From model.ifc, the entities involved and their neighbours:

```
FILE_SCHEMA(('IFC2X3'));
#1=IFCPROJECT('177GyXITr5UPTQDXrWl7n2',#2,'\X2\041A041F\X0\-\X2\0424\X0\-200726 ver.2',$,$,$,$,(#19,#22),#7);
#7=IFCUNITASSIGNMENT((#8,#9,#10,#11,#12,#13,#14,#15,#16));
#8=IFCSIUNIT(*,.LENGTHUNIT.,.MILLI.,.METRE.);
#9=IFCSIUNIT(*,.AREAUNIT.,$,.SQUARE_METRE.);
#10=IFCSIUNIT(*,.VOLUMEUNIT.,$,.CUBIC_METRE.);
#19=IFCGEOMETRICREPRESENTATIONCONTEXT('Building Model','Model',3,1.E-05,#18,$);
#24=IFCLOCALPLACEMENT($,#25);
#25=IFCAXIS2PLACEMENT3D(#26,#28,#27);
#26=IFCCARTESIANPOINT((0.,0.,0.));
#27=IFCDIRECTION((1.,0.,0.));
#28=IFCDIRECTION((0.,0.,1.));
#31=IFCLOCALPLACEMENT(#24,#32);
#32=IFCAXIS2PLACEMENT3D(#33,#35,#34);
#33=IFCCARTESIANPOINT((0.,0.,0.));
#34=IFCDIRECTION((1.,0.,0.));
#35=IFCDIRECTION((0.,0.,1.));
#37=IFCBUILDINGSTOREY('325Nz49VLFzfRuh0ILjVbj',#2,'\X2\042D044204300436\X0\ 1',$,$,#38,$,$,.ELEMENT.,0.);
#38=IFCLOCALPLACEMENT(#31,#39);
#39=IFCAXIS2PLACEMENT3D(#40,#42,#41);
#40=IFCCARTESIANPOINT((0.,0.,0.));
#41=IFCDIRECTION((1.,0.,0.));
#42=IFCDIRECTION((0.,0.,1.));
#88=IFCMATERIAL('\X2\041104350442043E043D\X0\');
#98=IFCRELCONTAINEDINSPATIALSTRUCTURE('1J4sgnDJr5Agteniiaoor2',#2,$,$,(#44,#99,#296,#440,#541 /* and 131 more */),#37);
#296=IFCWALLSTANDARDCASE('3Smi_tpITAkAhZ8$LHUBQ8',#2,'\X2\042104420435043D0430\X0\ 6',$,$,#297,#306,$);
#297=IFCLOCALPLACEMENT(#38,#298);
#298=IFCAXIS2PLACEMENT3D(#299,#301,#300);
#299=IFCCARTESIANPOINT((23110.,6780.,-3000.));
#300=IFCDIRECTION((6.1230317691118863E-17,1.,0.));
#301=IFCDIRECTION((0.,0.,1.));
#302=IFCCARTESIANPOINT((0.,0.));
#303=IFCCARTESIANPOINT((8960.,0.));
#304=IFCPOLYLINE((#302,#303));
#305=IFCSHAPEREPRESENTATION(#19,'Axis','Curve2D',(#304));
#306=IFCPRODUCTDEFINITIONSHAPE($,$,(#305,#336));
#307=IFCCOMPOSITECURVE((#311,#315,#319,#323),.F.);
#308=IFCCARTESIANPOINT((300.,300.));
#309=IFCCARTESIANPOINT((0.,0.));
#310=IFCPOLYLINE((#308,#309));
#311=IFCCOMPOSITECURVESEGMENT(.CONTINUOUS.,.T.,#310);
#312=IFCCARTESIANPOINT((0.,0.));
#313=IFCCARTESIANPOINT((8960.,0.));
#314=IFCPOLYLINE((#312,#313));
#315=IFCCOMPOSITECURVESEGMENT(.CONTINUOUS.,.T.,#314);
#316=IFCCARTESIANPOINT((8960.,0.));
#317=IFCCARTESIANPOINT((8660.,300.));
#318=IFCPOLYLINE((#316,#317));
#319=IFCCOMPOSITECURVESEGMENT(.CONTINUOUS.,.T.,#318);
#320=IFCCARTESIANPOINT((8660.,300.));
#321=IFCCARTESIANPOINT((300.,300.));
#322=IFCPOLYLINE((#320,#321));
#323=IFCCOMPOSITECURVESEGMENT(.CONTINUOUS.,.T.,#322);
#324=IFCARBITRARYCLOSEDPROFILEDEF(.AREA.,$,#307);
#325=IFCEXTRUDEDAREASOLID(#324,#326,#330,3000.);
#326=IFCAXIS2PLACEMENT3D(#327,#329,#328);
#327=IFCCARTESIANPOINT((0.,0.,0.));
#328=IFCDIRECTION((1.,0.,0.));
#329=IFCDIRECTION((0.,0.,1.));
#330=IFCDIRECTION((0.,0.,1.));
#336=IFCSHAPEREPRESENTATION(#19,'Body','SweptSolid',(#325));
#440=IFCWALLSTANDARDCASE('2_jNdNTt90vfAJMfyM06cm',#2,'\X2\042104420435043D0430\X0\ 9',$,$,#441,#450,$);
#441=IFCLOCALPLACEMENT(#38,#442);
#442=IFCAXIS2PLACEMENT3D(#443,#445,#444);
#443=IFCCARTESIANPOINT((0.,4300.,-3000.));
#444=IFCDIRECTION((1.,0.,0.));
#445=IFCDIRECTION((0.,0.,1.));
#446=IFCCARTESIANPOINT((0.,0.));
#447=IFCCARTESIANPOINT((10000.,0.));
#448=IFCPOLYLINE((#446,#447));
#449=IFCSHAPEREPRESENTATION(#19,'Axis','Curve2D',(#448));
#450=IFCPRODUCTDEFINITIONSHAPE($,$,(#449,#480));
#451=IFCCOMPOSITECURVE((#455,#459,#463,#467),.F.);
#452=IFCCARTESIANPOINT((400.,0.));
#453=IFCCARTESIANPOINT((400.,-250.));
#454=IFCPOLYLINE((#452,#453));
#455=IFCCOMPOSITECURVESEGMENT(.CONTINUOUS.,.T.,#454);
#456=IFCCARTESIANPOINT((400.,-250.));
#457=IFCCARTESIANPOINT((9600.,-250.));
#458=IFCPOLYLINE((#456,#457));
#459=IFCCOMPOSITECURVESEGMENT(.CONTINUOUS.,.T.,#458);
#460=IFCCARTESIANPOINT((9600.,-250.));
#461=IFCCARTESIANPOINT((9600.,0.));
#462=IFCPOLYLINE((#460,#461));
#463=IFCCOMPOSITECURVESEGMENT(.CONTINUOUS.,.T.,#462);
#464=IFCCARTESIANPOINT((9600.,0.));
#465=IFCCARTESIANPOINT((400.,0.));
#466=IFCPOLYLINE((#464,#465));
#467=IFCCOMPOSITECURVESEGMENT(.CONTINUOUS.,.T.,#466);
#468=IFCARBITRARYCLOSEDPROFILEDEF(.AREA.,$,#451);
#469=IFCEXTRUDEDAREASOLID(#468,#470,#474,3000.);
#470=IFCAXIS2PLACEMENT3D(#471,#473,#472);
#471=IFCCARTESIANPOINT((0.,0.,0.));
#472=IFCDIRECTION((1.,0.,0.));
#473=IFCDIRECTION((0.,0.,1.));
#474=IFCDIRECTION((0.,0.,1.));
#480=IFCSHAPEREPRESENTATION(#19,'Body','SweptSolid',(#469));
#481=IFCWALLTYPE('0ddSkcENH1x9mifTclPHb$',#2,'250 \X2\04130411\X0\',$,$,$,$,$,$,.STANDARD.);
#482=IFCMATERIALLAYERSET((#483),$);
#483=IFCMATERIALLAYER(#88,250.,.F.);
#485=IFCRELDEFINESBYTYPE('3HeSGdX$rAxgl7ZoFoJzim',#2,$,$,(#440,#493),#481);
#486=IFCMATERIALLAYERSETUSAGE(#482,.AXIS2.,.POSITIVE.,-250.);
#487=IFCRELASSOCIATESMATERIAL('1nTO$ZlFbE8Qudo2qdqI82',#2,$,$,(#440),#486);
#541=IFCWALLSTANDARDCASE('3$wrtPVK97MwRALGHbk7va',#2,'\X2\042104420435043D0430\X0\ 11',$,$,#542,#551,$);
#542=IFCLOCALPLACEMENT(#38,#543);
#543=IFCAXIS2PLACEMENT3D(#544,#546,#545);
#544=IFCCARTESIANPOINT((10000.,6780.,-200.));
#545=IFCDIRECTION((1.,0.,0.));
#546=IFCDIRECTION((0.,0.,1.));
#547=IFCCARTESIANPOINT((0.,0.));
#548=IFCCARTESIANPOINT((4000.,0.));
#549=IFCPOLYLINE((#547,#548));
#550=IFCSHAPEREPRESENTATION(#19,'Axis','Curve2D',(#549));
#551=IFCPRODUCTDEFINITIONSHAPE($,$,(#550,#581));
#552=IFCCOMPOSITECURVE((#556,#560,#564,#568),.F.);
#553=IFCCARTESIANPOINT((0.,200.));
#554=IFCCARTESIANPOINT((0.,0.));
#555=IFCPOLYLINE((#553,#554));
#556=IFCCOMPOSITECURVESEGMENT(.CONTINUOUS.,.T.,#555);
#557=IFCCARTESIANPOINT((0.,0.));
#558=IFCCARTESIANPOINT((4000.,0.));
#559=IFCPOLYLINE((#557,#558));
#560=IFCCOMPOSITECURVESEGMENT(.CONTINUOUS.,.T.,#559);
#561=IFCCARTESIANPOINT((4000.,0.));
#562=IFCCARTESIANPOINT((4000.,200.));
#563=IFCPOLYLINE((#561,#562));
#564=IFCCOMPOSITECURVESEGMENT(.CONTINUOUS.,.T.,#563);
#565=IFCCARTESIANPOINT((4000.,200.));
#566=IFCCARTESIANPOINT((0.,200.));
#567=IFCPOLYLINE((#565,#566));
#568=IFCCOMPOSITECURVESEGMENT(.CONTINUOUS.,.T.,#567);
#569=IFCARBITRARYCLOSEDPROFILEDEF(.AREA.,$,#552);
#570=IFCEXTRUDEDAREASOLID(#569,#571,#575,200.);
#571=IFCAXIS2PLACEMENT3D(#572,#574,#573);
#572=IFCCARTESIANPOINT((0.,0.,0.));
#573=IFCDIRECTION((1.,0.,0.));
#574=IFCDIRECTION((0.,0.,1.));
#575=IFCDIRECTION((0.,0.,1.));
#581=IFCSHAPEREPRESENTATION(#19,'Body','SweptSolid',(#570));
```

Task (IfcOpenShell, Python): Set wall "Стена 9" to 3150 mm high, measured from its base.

```python
import ifcopenshell
import ifcopenshell.geom
import ifcopenshell.util.shape
import ifcopenshell.util.unit

model = ifcopenshell.open("model.ifc")
unit_scale = ifcopenshell.util.unit.calculate_unit_scale(model)
settings = ifcopenshell.geom.settings()


def volume(element):
    """Net volume in cubic metres, openings subtracted."""
    shape = ifcopenshell.geom.create_shape(settings, element)
    return ifcopenshell.util.shape.get_volume(shape.geometry)


wall = model.by_id(440)
before = volume(wall)

body = next(r for r in wall.Representation.Representations if r.RepresentationIdentifier == "Body")
solid = body.Items[0]
old_height = solid.Depth
solid.Depth = 3.15 / unit_scale
after = volume(wall)

print(f"height {old_height:g} -> {solid.Depth:g}, volume {before:.3f} -> {after:.3f} m3")

model.write("model-out.ifc")
```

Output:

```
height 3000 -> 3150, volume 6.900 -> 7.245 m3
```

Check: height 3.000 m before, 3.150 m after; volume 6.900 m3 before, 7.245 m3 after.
